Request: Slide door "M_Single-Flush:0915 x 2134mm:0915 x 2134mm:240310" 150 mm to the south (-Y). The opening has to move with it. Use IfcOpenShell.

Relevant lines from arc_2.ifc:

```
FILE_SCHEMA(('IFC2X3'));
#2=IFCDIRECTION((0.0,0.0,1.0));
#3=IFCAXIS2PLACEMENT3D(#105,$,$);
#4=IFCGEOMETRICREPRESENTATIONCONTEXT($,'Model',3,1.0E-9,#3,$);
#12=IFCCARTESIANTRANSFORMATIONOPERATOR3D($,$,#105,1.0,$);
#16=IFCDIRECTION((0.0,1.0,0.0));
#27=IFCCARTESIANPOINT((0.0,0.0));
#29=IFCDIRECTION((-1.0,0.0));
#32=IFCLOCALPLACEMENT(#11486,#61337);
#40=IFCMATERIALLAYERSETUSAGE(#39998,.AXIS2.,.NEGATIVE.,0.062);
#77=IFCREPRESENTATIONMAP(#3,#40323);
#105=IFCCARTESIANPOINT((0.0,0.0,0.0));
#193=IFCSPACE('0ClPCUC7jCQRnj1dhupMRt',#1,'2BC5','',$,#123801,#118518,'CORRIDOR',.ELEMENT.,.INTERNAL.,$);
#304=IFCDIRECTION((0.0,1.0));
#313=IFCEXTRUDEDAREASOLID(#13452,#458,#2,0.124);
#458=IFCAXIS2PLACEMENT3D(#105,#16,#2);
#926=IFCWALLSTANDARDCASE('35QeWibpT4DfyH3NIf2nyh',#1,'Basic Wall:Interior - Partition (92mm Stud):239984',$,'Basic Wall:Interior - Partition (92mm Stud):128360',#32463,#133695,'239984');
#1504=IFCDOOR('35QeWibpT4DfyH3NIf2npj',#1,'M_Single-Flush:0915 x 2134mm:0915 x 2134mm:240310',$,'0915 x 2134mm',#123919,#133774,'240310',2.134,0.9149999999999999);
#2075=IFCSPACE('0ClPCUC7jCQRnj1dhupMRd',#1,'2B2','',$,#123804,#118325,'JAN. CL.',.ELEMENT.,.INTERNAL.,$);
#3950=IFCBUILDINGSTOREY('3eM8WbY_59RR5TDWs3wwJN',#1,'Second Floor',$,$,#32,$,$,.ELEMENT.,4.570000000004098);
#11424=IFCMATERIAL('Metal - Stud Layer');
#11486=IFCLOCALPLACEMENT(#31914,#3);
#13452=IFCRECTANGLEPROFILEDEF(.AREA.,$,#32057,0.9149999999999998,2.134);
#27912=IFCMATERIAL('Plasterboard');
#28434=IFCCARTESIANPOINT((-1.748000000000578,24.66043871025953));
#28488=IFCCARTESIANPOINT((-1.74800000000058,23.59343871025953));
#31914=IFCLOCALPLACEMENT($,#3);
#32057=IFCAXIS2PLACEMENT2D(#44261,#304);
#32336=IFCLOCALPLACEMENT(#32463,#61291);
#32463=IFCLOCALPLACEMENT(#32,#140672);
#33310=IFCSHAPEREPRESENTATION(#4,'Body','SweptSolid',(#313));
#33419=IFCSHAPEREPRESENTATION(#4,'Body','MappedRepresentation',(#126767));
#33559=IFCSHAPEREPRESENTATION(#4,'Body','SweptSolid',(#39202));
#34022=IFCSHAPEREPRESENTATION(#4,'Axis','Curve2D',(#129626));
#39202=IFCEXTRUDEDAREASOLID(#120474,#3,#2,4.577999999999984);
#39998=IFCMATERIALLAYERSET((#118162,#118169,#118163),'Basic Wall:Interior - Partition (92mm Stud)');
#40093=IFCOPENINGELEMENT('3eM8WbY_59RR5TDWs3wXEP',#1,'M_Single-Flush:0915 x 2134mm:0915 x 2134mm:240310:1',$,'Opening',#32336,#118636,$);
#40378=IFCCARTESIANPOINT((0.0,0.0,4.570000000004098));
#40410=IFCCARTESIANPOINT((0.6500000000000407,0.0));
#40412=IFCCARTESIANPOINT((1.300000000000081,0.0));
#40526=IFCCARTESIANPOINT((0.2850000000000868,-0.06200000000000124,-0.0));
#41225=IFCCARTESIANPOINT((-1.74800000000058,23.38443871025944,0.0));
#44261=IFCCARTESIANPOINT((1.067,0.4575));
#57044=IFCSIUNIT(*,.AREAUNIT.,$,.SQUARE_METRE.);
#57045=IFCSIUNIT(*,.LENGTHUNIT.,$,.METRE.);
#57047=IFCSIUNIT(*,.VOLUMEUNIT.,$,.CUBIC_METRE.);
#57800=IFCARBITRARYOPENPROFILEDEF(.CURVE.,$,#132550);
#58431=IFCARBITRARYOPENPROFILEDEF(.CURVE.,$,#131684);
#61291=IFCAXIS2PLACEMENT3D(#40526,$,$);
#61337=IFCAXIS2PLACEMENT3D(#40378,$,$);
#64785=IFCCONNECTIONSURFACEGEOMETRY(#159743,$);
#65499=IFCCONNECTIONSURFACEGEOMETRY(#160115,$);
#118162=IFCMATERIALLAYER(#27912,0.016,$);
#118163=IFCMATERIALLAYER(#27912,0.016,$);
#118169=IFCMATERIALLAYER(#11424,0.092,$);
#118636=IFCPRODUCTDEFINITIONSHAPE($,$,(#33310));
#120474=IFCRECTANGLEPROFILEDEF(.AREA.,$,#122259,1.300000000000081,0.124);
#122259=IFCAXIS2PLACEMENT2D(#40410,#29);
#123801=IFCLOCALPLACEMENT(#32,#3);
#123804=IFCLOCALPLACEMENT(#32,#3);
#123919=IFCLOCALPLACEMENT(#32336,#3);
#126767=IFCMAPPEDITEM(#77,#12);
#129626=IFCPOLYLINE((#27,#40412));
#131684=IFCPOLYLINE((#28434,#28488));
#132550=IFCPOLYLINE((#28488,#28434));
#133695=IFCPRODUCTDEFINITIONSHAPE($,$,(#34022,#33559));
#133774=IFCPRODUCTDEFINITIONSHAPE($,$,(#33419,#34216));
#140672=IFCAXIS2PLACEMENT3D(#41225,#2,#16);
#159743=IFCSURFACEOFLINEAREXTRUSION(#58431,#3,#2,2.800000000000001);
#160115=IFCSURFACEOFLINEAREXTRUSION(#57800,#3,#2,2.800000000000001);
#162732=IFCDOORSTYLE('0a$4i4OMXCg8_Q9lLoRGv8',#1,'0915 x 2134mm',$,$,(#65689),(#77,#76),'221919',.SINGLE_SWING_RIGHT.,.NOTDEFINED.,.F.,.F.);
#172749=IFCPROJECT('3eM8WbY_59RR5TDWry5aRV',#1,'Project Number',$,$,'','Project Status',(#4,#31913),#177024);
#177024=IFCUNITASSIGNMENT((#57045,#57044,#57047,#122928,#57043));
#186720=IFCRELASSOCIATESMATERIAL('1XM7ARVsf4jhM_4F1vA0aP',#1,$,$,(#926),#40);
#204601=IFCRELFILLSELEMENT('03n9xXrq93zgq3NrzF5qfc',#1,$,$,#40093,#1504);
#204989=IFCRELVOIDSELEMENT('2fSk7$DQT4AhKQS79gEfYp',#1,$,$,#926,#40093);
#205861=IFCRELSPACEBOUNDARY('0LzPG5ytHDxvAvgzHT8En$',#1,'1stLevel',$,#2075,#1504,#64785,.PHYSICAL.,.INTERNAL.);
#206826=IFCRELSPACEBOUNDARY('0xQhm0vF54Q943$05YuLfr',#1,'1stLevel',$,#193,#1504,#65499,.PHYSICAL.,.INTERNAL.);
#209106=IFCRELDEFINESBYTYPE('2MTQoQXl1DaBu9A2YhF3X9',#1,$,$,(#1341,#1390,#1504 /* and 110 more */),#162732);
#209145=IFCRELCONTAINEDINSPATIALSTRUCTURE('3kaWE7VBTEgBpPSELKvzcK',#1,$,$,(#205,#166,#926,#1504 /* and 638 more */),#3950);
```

```python
import numpy as np
import ifcopenshell
import ifcopenshell.api.geometry
import ifcopenshell.util.placement

model = ifcopenshell.open("arc_2.ifc")

door = model.by_id(1504)
opening = door.FillsVoids[0].RelatingOpeningElement
wall = opening.VoidsElements[0].RelatingBuildingElement

wall_matrix = ifcopenshell.util.placement.get_local_placement(wall.ObjectPlacement)
shift = wall_matrix[:3, 0] * -0.15
before = ifcopenshell.util.placement.get_local_placement(door.ObjectPlacement)[:3, 3].copy()

# The door is placed relative to its opening, so it follows when the opening moves.
matrix = ifcopenshell.util.placement.get_local_placement(opening.ObjectPlacement)
matrix[:3, 3] += shift
ifcopenshell.api.geometry.edit_object_placement(
    model, product=opening, matrix=matrix, is_si=False, should_transform_children=True
)

# Space boundary surfaces are stored in each space's coordinates; move them too.
for rel in door.ProvidesBoundaries:
    if not rel.ConnectionGeometry:
        continue
    surface = rel.ConnectionGeometry.SurfaceOnRelatingElement
    space_matrix = ifcopenshell.util.placement.get_local_placement(rel.RelatingSpace.ObjectPlacement)
    point = np.array(surface.Position.Location.Coordinates) + space_matrix[:3, :3].T @ shift
    surface.Position = model.createIfcAxis2Placement3D(
        model.createIfcCartesianPoint(point.tolist()), surface.Position.Axis, surface.Position.RefDirection
    )

after = ifcopenshell.util.placement.get_local_placement(door.ObjectPlacement)[:3, 3]
print("door moved by", (after - before).round(3) + 0.0)

model.write("arc_2-out.ifc")
```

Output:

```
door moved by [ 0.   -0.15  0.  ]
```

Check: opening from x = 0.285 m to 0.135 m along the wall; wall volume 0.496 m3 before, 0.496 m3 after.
